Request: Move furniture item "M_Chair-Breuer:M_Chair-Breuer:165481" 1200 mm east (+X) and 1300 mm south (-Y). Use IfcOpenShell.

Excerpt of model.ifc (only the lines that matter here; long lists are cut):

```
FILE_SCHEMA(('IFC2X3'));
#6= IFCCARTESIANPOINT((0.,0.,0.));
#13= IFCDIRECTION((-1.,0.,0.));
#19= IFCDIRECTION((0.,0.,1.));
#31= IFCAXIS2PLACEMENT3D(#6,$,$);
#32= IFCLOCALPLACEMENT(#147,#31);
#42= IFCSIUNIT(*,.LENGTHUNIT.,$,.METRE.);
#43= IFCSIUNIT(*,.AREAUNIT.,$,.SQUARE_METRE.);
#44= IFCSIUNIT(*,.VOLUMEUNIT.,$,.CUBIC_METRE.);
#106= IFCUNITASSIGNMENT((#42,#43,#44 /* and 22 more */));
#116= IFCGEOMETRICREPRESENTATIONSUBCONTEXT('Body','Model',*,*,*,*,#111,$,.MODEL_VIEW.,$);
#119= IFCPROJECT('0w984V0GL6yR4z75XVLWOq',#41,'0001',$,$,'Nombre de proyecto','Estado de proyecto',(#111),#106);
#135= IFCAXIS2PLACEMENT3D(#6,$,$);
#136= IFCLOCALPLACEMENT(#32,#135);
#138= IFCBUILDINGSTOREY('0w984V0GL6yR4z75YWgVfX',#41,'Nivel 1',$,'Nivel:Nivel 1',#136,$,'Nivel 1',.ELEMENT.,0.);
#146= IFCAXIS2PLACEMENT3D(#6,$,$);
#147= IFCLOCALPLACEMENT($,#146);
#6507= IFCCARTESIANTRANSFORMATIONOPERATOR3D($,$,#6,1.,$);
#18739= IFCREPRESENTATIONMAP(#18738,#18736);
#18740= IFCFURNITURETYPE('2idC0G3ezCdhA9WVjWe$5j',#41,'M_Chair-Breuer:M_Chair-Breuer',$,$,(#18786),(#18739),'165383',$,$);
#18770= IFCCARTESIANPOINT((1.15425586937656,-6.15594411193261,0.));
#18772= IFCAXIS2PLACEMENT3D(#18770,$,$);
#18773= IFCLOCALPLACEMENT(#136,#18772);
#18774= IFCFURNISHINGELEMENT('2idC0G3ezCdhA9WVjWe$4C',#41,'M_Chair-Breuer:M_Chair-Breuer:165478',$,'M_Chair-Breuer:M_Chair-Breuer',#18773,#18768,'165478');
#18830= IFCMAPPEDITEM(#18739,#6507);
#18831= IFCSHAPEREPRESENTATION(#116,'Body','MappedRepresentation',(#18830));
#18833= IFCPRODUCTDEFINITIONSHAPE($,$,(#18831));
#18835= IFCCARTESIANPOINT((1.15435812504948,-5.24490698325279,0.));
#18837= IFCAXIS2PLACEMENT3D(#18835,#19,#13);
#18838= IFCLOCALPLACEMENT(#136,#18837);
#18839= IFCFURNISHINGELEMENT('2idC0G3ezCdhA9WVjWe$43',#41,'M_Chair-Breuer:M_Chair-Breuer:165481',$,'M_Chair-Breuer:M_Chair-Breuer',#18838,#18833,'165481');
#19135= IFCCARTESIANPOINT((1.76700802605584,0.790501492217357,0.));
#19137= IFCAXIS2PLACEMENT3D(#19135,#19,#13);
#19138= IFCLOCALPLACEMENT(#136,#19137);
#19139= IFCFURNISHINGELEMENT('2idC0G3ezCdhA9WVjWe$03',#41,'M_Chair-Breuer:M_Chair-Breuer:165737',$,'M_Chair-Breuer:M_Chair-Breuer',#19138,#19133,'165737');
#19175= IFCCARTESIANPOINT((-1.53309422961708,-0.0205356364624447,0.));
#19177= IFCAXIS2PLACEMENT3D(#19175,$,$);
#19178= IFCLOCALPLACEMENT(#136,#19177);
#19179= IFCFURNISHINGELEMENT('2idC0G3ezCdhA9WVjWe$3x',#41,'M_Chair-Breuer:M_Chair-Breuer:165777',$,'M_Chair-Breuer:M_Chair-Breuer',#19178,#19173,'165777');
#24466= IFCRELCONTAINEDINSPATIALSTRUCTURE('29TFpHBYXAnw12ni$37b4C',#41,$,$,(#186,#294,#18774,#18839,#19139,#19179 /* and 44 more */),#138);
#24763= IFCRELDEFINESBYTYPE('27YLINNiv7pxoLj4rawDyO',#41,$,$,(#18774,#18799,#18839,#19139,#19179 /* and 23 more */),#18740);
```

```python
import ifcopenshell
import ifcopenshell.api.geometry
import ifcopenshell.util.placement

model = ifcopenshell.open("model.ifc")

item = model.by_id(18839)
matrix = ifcopenshell.util.placement.get_local_placement(item.ObjectPlacement)
matrix[0, 3] += 1.2
matrix[1, 3] -= 1.3
ifcopenshell.api.geometry.edit_object_placement(model, product=item, matrix=matrix, is_si=False)

print(ifcopenshell.util.placement.get_local_placement(item.ObjectPlacement).round(3) + 0.0)

model.write("model_rev.ifc")
```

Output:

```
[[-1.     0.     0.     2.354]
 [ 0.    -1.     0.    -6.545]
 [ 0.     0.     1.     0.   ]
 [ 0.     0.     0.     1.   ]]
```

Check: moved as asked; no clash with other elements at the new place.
